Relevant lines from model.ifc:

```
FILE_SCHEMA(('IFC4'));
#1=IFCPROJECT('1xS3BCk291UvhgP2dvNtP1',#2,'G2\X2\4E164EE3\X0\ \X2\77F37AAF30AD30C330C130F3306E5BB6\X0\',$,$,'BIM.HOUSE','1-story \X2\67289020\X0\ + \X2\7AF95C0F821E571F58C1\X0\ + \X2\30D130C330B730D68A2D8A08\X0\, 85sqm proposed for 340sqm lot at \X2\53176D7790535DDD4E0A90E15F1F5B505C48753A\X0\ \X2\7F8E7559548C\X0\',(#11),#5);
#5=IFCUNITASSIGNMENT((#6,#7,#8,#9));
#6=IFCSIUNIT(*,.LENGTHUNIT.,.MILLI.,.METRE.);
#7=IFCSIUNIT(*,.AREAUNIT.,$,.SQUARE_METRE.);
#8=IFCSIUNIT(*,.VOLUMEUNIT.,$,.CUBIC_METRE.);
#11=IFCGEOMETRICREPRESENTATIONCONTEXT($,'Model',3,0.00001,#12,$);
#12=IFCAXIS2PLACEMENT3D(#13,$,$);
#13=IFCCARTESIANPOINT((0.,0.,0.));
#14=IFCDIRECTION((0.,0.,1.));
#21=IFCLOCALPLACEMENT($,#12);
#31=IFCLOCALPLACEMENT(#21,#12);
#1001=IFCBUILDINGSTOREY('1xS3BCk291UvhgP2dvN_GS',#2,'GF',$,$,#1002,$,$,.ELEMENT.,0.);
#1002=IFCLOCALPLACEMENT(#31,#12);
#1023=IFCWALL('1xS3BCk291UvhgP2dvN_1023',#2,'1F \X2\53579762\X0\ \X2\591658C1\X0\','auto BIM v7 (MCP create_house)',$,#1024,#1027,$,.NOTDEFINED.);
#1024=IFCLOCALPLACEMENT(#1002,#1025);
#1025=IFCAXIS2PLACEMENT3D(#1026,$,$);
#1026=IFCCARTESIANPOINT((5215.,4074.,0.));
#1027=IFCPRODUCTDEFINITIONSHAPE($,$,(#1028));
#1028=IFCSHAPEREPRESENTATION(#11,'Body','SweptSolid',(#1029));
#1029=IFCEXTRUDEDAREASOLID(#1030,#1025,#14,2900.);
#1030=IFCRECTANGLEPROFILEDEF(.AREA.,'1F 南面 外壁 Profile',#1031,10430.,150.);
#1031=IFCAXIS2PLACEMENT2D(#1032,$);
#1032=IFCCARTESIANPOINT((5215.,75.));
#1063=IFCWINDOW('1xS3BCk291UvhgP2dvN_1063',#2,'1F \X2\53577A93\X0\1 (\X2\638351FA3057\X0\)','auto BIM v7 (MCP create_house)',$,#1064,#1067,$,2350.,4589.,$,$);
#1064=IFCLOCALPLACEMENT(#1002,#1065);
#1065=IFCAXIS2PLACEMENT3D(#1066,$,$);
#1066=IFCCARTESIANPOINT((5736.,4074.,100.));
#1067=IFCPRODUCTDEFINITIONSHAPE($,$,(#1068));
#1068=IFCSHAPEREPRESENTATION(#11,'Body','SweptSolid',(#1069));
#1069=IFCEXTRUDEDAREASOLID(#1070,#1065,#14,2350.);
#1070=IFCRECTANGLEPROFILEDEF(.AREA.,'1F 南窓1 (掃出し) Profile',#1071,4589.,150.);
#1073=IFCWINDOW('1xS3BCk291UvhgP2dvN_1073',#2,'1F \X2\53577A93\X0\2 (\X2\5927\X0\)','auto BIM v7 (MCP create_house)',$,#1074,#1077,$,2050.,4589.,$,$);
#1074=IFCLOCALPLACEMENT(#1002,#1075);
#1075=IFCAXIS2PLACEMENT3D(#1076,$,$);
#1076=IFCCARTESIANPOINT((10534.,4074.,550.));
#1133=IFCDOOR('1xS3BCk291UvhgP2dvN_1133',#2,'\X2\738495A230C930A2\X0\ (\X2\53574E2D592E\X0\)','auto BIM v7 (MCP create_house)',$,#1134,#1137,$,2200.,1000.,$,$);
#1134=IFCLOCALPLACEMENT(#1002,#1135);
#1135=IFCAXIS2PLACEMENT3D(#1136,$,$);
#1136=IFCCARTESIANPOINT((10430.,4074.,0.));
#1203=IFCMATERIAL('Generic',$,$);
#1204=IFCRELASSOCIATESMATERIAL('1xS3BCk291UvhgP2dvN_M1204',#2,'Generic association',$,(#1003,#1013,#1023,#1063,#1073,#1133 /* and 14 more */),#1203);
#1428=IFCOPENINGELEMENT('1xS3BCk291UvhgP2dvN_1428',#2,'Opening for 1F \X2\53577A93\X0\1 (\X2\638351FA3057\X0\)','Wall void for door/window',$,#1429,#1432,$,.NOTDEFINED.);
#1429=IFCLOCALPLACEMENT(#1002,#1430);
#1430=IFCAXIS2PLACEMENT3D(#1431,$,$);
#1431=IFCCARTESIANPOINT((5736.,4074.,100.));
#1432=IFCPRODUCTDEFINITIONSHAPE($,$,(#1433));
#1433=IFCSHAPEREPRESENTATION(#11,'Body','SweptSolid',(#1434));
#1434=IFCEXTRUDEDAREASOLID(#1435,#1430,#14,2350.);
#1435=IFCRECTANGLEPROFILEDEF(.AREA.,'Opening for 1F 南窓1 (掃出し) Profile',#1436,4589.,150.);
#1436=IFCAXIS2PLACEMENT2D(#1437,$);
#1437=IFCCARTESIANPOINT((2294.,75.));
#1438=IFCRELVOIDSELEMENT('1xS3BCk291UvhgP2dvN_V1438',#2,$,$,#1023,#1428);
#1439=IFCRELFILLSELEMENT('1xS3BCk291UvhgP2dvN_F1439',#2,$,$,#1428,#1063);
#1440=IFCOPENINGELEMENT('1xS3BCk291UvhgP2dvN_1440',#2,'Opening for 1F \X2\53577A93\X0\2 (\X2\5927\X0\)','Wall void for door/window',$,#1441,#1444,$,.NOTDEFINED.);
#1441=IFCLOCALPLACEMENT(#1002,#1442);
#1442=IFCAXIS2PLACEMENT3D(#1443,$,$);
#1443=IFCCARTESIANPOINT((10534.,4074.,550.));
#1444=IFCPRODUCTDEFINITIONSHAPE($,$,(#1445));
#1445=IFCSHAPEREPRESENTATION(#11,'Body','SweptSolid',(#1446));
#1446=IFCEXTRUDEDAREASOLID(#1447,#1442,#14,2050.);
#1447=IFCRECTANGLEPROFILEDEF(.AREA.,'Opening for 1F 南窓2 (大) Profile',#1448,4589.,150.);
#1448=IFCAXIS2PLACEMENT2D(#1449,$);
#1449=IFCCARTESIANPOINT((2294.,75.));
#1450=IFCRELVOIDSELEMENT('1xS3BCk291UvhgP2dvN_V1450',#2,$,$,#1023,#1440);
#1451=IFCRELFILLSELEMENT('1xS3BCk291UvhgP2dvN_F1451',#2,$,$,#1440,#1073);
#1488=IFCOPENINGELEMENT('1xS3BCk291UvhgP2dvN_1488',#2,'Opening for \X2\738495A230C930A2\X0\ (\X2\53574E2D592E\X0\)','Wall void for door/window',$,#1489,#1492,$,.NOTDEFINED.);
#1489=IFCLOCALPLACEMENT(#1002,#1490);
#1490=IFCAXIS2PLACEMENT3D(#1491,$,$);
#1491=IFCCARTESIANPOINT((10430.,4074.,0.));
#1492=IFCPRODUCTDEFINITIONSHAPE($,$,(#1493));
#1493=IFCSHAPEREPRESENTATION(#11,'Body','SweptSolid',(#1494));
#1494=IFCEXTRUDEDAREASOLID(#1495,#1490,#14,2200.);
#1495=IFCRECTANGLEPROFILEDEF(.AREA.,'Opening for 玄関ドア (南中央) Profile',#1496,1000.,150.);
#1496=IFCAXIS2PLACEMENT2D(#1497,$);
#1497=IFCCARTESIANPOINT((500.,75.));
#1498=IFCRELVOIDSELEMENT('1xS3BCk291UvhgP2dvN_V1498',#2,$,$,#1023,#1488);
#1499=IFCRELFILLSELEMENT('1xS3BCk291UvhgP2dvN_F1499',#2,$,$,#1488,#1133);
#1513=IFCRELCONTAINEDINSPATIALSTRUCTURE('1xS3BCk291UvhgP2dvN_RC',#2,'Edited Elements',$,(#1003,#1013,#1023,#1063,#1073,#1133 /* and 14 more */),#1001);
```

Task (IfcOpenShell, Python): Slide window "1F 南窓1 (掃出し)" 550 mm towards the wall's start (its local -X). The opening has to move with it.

```python
import ifcopenshell
import ifcopenshell.api.geometry
import ifcopenshell.util.placement

model = ifcopenshell.open("model.ifc")

window = model.by_guid("1xS3BCk291UvhgP2dvN_1063")
opening = window.FillsVoids[0].RelatingOpeningElement
wall = opening.VoidsElements[0].RelatingBuildingElement

wall_matrix = ifcopenshell.util.placement.get_local_placement(wall.ObjectPlacement)
shift = wall_matrix[:3, 0] * -550.0
before = ifcopenshell.util.placement.get_local_placement(window.ObjectPlacement)[:3, 3].copy()

# The window is not placed relative to its opening, so move both.
for product in (opening, window):
    matrix = ifcopenshell.util.placement.get_local_placement(product.ObjectPlacement)
    matrix[:3, 3] += shift
    ifcopenshell.api.geometry.edit_object_placement(model, product=product, matrix=matrix, is_si=False)

after = ifcopenshell.util.placement.get_local_placement(window.ObjectPlacement)[:3, 3]
print("window moved by", (after - before).round(3) + 0.0)

model.write("model_v2.ifc")
```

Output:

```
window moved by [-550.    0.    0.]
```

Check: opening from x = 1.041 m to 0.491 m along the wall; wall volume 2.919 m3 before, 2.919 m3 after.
